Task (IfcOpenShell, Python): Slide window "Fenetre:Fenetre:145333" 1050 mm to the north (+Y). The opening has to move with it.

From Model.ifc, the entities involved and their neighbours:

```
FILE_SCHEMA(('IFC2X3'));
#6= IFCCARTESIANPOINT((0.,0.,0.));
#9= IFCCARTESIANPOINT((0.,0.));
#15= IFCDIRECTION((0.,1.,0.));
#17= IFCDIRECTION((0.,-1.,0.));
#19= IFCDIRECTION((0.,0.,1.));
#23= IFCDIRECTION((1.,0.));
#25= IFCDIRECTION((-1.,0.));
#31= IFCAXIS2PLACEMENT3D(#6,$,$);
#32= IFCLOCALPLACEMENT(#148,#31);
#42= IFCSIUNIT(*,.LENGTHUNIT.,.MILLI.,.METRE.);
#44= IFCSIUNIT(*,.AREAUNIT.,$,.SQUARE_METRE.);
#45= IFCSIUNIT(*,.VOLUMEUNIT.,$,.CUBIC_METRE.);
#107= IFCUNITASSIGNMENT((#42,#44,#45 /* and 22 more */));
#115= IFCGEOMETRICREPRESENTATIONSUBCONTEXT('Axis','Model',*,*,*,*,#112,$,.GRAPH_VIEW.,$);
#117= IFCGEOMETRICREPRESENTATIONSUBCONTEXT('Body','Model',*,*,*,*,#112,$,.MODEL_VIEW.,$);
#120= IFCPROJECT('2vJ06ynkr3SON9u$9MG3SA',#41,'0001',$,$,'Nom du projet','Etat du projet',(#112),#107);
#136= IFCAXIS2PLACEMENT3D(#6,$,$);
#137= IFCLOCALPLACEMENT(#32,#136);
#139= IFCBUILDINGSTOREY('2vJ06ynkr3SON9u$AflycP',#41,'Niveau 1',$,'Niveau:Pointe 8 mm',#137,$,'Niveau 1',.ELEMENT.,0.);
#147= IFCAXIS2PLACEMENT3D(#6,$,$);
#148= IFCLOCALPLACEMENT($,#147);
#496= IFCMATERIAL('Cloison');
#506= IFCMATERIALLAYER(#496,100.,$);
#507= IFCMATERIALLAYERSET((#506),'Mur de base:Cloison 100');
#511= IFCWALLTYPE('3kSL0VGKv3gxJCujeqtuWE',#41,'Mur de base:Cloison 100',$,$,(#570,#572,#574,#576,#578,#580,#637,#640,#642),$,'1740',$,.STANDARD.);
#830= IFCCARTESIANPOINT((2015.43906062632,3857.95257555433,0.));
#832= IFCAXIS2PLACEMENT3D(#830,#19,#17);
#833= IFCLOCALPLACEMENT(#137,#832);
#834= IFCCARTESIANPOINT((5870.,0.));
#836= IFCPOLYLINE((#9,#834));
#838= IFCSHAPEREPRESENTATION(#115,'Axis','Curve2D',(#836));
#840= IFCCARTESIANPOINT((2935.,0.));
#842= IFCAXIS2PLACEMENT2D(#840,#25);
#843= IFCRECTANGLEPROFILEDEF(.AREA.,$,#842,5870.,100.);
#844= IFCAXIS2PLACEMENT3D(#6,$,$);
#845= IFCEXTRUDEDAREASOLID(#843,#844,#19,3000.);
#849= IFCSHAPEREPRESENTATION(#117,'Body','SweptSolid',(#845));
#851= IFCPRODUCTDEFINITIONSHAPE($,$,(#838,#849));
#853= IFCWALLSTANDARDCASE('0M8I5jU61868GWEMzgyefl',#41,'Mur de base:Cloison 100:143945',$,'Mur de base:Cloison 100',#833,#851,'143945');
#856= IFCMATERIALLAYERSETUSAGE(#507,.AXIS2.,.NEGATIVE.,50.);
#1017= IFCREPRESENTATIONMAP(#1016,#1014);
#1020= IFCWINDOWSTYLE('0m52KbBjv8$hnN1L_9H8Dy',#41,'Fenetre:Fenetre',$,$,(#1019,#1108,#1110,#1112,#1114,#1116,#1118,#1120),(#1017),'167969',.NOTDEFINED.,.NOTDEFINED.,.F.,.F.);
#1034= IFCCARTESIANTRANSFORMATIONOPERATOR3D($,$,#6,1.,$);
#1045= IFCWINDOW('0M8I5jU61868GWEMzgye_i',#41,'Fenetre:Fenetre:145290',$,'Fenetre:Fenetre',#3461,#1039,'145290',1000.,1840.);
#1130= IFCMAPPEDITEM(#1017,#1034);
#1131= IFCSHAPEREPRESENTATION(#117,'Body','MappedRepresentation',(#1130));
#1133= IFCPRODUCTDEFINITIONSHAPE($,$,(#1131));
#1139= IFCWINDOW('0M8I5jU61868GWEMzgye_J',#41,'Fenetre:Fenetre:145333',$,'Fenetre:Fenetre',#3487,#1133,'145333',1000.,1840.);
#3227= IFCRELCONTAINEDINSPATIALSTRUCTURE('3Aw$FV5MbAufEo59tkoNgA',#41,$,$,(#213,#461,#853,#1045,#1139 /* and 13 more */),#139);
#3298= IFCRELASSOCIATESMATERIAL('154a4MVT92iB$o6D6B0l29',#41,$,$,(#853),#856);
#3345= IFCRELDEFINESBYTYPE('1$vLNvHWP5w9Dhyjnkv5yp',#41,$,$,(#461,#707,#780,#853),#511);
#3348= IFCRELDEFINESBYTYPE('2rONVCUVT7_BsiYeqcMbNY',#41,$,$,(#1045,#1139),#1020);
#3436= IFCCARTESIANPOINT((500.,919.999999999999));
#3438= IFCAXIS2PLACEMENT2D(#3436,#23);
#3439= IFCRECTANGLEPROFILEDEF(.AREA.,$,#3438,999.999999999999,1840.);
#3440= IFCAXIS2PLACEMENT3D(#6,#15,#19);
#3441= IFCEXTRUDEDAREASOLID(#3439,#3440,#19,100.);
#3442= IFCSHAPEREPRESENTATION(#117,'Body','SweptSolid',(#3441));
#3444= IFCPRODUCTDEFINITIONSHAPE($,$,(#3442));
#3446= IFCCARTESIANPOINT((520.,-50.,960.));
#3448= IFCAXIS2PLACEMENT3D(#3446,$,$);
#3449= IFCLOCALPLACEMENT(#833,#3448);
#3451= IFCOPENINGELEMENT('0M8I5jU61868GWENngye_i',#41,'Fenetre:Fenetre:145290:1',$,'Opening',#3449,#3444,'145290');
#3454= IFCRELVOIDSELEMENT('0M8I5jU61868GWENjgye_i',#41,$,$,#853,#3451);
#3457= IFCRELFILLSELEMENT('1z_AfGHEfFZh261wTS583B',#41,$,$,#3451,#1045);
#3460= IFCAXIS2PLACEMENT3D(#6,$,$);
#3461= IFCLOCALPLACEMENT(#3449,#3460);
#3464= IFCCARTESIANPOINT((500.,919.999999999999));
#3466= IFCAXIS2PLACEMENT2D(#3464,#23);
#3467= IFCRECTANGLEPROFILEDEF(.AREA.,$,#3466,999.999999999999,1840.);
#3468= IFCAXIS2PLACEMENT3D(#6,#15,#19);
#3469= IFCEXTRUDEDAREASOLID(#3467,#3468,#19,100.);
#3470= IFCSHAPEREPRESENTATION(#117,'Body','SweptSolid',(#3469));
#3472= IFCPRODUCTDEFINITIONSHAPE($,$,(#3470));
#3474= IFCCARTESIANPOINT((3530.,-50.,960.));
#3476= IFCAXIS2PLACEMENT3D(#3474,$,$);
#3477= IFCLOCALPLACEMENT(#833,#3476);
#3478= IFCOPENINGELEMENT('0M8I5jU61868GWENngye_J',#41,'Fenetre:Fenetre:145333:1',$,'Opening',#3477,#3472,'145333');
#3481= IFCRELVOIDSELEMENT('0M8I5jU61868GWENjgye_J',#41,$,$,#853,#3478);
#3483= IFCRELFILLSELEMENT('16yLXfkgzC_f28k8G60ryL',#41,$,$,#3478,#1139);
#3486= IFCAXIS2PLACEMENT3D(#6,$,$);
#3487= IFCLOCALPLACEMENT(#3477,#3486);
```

```python
import ifcopenshell
import ifcopenshell.api.geometry
import ifcopenshell.util.placement
import ifcopenshell.util.unit

model = ifcopenshell.open("Model.ifc")
unit_scale = ifcopenshell.util.unit.calculate_unit_scale(model)

window = model.by_guid("0M8I5jU61868GWEMzgye_J")
opening = window.FillsVoids[0].RelatingOpeningElement
wall = opening.VoidsElements[0].RelatingBuildingElement

wall_matrix = ifcopenshell.util.placement.get_local_placement(wall.ObjectPlacement)
shift = wall_matrix[:3, 0] * -1.05 / unit_scale
before = ifcopenshell.util.placement.get_local_placement(window.ObjectPlacement)[:3, 3].copy()

# The window is placed relative to its opening, so it follows when the opening moves.
matrix = ifcopenshell.util.placement.get_local_placement(opening.ObjectPlacement)
matrix[:3, 3] += shift
ifcopenshell.api.geometry.edit_object_placement(
    model, product=opening, matrix=matrix, is_si=False, should_transform_children=True
)

after = ifcopenshell.util.placement.get_local_placement(window.ObjectPlacement)[:3, 3]
print("window moved by", (after - before).round(3) + 0.0)

model.write("Model-out.ifc")
```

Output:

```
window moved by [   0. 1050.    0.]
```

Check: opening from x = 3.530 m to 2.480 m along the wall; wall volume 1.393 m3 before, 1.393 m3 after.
